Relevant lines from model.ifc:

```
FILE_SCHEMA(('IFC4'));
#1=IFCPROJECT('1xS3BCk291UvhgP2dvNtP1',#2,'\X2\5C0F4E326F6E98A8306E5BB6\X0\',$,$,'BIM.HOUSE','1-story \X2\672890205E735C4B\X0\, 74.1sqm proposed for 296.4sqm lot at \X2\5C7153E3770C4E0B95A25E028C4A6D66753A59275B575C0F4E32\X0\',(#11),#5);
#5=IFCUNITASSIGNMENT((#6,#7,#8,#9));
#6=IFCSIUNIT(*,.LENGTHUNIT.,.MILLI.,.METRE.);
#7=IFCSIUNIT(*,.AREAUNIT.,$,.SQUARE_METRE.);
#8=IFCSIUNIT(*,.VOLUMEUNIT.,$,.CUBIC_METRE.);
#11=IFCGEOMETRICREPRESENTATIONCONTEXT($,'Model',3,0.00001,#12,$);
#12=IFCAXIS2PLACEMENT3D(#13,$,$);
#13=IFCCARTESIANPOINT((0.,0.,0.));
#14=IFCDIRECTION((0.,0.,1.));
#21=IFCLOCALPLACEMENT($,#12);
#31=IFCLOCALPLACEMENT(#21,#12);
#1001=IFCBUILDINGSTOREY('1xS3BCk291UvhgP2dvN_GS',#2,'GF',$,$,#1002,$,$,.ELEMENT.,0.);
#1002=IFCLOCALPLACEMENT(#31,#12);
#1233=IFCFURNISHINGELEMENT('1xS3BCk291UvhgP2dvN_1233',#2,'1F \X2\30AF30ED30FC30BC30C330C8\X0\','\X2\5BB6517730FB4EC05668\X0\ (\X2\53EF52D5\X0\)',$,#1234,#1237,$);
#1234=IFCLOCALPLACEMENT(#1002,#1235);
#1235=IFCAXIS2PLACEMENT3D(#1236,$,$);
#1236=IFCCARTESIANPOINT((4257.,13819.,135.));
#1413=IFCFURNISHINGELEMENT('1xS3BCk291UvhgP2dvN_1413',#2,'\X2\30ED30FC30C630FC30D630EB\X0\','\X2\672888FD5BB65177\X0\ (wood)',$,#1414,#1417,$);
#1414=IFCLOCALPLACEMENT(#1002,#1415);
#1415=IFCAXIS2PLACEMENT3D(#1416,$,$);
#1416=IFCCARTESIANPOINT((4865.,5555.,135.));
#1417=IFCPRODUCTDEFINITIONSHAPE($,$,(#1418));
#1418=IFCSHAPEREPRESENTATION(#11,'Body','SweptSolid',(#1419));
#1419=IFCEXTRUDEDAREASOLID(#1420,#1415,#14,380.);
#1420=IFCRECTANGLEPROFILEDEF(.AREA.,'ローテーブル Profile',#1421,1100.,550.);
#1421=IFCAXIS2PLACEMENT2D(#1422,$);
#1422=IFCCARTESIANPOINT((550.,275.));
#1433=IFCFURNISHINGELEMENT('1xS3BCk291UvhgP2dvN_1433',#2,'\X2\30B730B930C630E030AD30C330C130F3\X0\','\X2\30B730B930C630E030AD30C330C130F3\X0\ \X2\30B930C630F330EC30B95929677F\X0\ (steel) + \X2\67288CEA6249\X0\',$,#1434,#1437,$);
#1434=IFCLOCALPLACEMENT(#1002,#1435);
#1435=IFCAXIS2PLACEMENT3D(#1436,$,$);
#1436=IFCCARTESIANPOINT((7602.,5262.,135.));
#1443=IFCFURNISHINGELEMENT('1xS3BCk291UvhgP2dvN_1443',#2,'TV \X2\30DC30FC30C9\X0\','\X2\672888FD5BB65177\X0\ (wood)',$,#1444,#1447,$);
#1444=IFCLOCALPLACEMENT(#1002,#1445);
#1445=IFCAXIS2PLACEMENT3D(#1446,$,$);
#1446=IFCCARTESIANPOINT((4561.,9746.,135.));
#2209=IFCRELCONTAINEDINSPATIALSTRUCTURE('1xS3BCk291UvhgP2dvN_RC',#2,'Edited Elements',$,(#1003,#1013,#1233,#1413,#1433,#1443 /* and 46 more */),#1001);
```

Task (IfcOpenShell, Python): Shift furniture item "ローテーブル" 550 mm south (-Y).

```python
import ifcopenshell
import ifcopenshell.api.geometry
import ifcopenshell.util.placement

model = ifcopenshell.open("model.ifc")

item = model.by_id(1413)
matrix = ifcopenshell.util.placement.get_local_placement(item.ObjectPlacement)
matrix[1, 3] -= 550.0
ifcopenshell.api.geometry.edit_object_placement(model, product=item, matrix=matrix, is_si=False)

print(ifcopenshell.util.placement.get_local_placement(item.ObjectPlacement).round(3) + 0.0)

model.write("model_v2.ifc")
```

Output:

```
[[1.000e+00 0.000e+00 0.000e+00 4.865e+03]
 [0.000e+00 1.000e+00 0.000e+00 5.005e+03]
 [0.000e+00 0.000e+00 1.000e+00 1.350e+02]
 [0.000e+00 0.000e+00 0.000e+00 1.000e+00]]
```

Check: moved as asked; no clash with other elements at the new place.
